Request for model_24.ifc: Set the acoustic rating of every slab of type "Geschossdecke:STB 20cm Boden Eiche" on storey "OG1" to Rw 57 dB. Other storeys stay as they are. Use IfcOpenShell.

First a look at what the model holds.

```python
import ifcopenshell
import ifcopenshell.util.element

model = ifcopenshell.open("model_24.ifc")
print(model.schema)
storey = next(s for s in model.by_type("IfcBuildingStorey") if s.Name == "OG1")
slabs = [e for e in ifcopenshell.util.element.get_decomposition(storey) if e.is_a("IfcSlab")]
seen = {}
for e in slabs:
    element_type = ifcopenshell.util.element.get_type(e)
    key = (element_type.Name if element_type != e and element_type else None, ifcopenshell.util.element.get_pset(e, "Pset_SlabCommon", "AcousticRating"))
    seen[key] = seen.get(key, 0) + 1
for (name, value), count in sorted(seen.items(), key=str):
    print(count, "x", name, "|", value)
```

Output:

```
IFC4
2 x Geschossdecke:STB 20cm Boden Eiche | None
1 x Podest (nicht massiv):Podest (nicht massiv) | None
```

```python
import ifcopenshell
import ifcopenshell.api.pset
import ifcopenshell.util.element

model = ifcopenshell.open("model_24.ifc")

storey = next(s for s in model.by_type("IfcBuildingStorey") if s.Name == "OG1")
slabs = [e for e in ifcopenshell.util.element.get_decomposition(storey) if e.is_a("IfcSlab")]

count = 0
for e in slabs:
    element_type = ifcopenshell.util.element.get_type(e)
    if element_type in (None, e) or element_type.Name != "Geschossdecke:STB 20cm Boden Eiche":
        continue
    # add_pset returns the element's existing set when there is one.
    pset = ifcopenshell.api.pset.add_pset(model, product=e, name="Pset_SlabCommon")
    ifcopenshell.api.pset.edit_pset(model, pset=pset, properties={"AcousticRating": "Rw 57 dB"})
    count += 1

print(count, "slabs updated")

model.write("model_24-out.ifc")
```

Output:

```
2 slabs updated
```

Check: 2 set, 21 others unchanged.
